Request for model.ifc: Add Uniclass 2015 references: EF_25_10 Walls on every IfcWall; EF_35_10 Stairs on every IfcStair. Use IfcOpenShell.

First a look at what the model holds.

```python
import ifcopenshell

model = ifcopenshell.open("model.ifc")
print(model.schema)
print("classifications:", [c.Name for c in model.by_type("IfcClassification")])
for ifc_class in ("IfcDoor", "IfcRoof", "IfcStair", "IfcWall", "IfcWindow"):
    print(ifc_class, len(model.by_type(ifc_class)))
```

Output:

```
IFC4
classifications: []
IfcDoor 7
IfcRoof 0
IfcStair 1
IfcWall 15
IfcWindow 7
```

```python
import ifcopenshell
import ifcopenshell.api.classification

model = ifcopenshell.open("model.ifc")

system = ifcopenshell.api.classification.add_classification(model, classification="Uniclass 2015")

codes = {
    "IfcWall": ("EF_25_10", "Walls"),
    "IfcStair": ("EF_35_10", "Stairs"),
}
for ifc_class, (code, name) in codes.items():
    products = model.by_type(ifc_class)
    ifcopenshell.api.classification.add_reference(
        model, products=products, classification=system, identification=code, name=name
    )
    print(code, len(products))

model.write("model-out.ifc")
```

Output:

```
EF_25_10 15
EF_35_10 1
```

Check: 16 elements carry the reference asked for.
